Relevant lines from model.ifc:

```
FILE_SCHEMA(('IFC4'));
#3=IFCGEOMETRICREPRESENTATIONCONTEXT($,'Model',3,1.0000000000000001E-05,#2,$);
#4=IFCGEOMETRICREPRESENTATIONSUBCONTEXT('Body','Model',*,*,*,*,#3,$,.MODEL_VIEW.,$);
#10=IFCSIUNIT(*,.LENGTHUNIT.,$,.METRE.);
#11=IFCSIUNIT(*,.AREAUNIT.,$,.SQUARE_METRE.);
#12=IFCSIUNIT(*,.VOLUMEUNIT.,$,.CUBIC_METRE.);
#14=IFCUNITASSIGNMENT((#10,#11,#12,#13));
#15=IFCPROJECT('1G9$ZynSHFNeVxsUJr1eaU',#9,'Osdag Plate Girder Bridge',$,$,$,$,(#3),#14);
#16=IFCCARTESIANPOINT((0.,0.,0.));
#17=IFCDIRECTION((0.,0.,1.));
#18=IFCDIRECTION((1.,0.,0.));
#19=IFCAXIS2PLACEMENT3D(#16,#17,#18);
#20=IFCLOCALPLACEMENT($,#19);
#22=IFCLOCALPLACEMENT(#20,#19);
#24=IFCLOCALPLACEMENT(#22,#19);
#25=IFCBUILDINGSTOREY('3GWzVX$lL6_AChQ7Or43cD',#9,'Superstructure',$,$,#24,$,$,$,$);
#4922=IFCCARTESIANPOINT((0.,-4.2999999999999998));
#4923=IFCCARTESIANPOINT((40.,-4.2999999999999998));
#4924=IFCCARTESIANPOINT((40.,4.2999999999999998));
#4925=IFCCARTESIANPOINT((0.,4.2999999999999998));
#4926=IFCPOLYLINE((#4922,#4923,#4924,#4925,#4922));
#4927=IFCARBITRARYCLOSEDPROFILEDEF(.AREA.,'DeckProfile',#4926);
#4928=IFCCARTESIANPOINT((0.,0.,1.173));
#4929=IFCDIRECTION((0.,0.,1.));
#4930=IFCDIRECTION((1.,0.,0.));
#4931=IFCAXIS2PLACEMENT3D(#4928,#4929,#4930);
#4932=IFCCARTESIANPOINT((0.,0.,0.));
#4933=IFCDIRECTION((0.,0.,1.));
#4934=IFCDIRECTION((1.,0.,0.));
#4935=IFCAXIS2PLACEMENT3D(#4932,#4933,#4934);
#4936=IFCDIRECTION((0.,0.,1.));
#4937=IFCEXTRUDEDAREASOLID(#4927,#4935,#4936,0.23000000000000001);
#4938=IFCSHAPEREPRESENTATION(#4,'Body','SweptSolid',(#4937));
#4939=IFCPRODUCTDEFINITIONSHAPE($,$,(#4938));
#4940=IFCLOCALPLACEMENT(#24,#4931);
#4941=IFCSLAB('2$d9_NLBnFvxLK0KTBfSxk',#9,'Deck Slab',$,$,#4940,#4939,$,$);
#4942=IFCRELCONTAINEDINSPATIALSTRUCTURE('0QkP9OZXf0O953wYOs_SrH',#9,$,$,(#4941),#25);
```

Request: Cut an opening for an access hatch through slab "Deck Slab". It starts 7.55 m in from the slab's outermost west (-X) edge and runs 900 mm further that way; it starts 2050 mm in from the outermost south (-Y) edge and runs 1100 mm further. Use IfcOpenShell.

```python
import numpy as np
import ifcopenshell
import ifcopenshell.api.feature
import ifcopenshell.api.geometry
import ifcopenshell.api.root
import ifcopenshell.geom
import ifcopenshell.util.placement
import ifcopenshell.util.representation
import ifcopenshell.util.shape
import ifcopenshell.util.unit

model = ifcopenshell.open("model.ifc")
unit_scale = ifcopenshell.util.unit.calculate_unit_scale(model)
settings = ifcopenshell.geom.settings()


def volume(element):
    """Net volume in cubic metres, openings subtracted."""
    shape = ifcopenshell.geom.create_shape(settings, element)
    return ifcopenshell.util.shape.get_volume(shape.geometry)


slab = model.by_guid("2$d9_NLBnFvxLK0KTBfSxk")
before = volume(slab)

# Extent in the slab's own axes, in metres. The edges named are its -X and -Y sides.
slab_shape = ifcopenshell.geom.create_shape(settings, slab)
vertices = ifcopenshell.util.shape.get_vertices(slab_shape.geometry)
x_min, y_min, bottom = vertices.min(axis=0)
top = vertices[:, 2].max()

opening = ifcopenshell.api.root.create_entity(model, ifc_class="IfcOpeningElement", name="Access hatch opening", predefined_type="OPENING")
context = ifcopenshell.util.representation.get_context(model, "Model", "Body", "MODEL_VIEW")
width, depth = 0.9, 1.1
outline = [(0.0, 0.0), (width, 0.0), (width, depth), (0.0, depth), (0.0, 0.0)]
# Overshoot both faces by 50 mm so the cut is clean.
shape = ifcopenshell.api.geometry.add_slab_representation(
    model, context=context, depth=top - bottom + 0.1, polyline=outline
)
ifcopenshell.api.geometry.assign_representation(model, product=opening, representation=shape)

matrix = ifcopenshell.util.placement.get_local_placement(slab.ObjectPlacement)
matrix[:, 3] = matrix @ np.append(np.array([x_min + 7.55, y_min + 2.05, bottom - 0.05]) / unit_scale, 1.0)
ifcopenshell.api.geometry.edit_object_placement(model, product=opening, matrix=matrix, is_si=False)
ifcopenshell.api.feature.add_feature(model, feature=opening, element=slab)

after = volume(slab)

print(f"slab volume {before:.3f} -> {after:.3f} m3")

model.write("model-out.ifc")
```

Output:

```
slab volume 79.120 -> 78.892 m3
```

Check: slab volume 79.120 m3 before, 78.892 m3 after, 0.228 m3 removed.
